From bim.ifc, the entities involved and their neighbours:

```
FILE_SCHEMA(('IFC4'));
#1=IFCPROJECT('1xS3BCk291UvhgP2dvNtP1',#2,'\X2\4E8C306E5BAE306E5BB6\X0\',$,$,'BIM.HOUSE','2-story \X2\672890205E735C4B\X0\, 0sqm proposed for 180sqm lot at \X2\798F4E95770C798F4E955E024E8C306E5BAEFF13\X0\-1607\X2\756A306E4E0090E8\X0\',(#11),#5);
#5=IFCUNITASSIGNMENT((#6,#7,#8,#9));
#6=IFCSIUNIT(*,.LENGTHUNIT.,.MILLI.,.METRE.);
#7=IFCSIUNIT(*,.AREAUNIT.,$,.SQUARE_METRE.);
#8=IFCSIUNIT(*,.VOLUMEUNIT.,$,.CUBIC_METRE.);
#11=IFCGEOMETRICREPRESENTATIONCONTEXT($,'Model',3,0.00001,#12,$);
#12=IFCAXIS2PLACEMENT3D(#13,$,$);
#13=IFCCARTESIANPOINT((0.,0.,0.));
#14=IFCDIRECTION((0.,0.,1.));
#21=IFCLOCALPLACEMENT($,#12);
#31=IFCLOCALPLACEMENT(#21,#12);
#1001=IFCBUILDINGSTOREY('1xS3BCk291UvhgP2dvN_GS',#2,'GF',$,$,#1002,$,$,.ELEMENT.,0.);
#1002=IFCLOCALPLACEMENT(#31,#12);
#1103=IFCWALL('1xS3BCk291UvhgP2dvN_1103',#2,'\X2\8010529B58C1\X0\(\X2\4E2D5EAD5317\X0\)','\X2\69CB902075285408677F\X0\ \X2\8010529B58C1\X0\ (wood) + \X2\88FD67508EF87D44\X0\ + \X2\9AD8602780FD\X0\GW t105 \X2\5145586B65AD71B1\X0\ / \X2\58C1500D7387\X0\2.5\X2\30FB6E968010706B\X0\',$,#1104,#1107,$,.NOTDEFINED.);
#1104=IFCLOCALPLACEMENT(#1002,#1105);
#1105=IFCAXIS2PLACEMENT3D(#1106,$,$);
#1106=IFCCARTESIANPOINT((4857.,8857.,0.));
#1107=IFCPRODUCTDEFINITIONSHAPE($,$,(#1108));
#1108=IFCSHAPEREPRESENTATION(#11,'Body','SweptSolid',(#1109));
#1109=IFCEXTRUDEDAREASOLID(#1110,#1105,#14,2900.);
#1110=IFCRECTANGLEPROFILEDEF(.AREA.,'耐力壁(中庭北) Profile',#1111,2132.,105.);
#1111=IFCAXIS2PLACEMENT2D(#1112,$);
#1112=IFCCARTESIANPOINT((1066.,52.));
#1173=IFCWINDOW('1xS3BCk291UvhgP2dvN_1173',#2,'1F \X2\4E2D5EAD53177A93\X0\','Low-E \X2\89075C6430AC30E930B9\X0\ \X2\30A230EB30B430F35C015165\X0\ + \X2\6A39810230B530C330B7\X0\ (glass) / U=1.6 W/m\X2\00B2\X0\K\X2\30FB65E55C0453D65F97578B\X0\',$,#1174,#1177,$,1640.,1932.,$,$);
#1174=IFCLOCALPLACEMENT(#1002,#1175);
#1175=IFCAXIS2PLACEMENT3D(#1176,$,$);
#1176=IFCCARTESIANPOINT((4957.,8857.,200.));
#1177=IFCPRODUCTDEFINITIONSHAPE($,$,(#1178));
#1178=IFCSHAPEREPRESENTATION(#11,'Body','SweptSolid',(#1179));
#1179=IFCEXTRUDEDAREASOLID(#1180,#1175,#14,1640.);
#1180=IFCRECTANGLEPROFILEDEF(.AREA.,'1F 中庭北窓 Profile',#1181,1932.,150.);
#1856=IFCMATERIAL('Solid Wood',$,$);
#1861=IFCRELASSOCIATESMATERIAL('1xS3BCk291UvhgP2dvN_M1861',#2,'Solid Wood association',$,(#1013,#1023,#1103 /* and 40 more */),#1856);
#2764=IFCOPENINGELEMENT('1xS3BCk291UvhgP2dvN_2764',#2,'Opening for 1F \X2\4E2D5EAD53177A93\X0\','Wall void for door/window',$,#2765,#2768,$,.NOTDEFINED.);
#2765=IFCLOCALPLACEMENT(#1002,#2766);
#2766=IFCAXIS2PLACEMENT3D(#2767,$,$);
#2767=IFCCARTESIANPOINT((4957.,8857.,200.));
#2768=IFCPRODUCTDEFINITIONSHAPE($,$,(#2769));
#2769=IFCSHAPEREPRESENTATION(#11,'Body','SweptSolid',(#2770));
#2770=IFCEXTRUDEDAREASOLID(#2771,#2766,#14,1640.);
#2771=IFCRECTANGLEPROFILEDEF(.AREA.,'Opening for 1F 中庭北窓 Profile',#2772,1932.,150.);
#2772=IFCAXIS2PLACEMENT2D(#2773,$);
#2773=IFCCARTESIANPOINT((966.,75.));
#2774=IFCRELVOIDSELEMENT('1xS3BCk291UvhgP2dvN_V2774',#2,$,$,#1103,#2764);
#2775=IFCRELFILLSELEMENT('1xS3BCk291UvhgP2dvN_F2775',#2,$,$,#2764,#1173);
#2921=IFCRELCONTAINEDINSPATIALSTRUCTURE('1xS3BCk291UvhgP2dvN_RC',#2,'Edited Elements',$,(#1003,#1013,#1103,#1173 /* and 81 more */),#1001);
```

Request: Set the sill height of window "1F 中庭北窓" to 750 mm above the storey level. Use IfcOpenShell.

```python
import numpy as np
import ifcopenshell
import ifcopenshell.api.geometry
import ifcopenshell.geom
import ifcopenshell.util.element
import ifcopenshell.util.placement
import ifcopenshell.util.shape
import ifcopenshell.util.unit

model = ifcopenshell.open("bim.ifc")
unit_scale = ifcopenshell.util.unit.calculate_unit_scale(model)

window = model.by_id(1173)
opening = window.FillsVoids[0].RelatingOpeningElement
storey = ifcopenshell.util.element.get_container(window, ifc_class="IfcBuildingStorey")
level = ifcopenshell.util.placement.get_local_placement(storey.ObjectPlacement)[2, 3]

# The opening's origin need not be at the sill, so measure its lowest point.
shape = ifcopenshell.geom.create_shape(ifcopenshell.geom.settings(), opening)
bottom = ifcopenshell.util.shape.get_shape_bottom_elevation(shape, shape.geometry) / unit_scale
dz = level + 0.75 / unit_scale - bottom

shift = np.array([0.0, 0.0, dz])
# The window is not placed relative to its opening, so move both.
for product in (opening, window):
    matrix = ifcopenshell.util.placement.get_local_placement(product.ObjectPlacement)
    matrix[:3, 3] += shift
    ifcopenshell.api.geometry.edit_object_placement(model, product=product, matrix=matrix, is_si=False)

print(f"moved by {dz * unit_scale:+.3f} m")

model.write("bim_rev.ifc")
```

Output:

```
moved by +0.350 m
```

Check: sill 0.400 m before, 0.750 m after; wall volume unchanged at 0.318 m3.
